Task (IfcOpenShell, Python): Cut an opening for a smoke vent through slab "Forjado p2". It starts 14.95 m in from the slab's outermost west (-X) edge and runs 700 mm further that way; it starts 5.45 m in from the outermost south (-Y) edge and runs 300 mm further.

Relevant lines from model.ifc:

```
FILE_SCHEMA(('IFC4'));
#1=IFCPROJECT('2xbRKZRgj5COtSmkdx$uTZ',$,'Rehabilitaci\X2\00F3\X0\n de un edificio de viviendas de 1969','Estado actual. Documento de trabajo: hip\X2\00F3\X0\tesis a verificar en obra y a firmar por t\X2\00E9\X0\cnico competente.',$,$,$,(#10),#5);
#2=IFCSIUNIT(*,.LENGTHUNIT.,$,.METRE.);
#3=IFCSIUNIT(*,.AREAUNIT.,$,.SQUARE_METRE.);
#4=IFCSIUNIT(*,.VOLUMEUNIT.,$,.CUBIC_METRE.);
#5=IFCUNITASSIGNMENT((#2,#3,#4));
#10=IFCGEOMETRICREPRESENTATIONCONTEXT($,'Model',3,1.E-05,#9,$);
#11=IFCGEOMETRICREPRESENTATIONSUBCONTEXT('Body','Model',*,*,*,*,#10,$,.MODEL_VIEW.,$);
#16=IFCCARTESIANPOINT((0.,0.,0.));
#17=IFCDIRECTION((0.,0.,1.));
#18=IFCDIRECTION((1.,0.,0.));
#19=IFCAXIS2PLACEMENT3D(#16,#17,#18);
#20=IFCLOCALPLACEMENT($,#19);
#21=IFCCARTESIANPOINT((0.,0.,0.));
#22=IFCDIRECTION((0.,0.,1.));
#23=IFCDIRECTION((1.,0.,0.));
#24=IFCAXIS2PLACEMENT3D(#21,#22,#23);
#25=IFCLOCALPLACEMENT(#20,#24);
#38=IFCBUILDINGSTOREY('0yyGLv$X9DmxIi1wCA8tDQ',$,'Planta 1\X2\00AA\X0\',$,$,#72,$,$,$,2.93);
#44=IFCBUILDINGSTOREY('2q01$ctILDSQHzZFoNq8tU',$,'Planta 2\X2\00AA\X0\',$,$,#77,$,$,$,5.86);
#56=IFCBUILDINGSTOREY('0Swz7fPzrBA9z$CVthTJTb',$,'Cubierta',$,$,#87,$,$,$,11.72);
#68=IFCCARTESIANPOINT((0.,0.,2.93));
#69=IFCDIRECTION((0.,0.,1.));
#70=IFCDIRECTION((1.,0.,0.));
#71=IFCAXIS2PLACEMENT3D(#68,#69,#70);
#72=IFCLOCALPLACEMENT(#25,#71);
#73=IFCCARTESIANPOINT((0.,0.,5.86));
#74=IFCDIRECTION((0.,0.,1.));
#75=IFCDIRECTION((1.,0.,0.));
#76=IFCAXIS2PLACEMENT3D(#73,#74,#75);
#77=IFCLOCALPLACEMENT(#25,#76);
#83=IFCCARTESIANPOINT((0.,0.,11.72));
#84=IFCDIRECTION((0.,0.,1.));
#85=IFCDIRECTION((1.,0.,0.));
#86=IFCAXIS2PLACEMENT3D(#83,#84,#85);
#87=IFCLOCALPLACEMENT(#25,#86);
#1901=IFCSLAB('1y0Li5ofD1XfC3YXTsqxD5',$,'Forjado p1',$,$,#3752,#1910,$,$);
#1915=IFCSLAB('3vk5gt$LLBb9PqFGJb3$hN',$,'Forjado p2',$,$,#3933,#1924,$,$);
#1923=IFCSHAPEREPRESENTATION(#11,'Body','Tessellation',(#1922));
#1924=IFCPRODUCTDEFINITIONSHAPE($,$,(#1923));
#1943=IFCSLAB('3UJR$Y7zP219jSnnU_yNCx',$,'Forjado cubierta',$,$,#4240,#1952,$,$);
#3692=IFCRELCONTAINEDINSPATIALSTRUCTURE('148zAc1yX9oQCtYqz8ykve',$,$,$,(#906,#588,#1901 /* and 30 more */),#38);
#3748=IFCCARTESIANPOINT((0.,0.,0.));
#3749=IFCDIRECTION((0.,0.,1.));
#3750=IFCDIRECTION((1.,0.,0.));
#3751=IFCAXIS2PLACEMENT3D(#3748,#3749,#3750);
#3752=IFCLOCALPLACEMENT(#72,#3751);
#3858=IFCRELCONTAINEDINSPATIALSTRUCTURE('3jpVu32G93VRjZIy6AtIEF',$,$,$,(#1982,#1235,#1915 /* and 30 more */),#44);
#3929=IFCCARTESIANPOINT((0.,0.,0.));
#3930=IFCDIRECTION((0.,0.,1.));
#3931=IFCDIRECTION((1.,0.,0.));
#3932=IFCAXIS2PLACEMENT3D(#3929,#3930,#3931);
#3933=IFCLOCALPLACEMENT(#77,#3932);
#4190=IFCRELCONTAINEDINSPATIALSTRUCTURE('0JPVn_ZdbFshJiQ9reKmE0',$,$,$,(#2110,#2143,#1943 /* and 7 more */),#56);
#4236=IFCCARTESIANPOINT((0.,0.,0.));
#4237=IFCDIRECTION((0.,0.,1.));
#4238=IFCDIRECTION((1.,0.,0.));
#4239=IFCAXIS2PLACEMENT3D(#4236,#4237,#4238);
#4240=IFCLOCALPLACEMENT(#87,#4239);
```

```python
import numpy as np
import ifcopenshell
import ifcopenshell.api.feature
import ifcopenshell.api.geometry
import ifcopenshell.api.root
import ifcopenshell.geom
import ifcopenshell.util.placement
import ifcopenshell.util.representation
import ifcopenshell.util.shape
import ifcopenshell.util.unit

model = ifcopenshell.open("model.ifc")
unit_scale = ifcopenshell.util.unit.calculate_unit_scale(model)
settings = ifcopenshell.geom.settings()


def volume(element):
    """Net volume in cubic metres, openings subtracted."""
    shape = ifcopenshell.geom.create_shape(settings, element)
    return ifcopenshell.util.shape.get_volume(shape.geometry)


slab = model.by_id(1915)
before = volume(slab)

# Extent in the slab's own axes, in metres. The edges named are its -X and -Y sides.
slab_shape = ifcopenshell.geom.create_shape(settings, slab)
vertices = ifcopenshell.util.shape.get_vertices(slab_shape.geometry)
x_min, y_min, bottom = vertices.min(axis=0)
top = vertices[:, 2].max()

opening = ifcopenshell.api.root.create_entity(model, ifc_class="IfcOpeningElement", name="Smoke vent opening", predefined_type="OPENING")
context = ifcopenshell.util.representation.get_context(model, "Model", "Body", "MODEL_VIEW")
width, depth = 0.7, 0.3
outline = [(0.0, 0.0), (width, 0.0), (width, depth), (0.0, depth), (0.0, 0.0)]
# Overshoot both faces by 50 mm so the cut is clean.
shape = ifcopenshell.api.geometry.add_slab_representation(
    model, context=context, depth=top - bottom + 0.1, polyline=outline
)
ifcopenshell.api.geometry.assign_representation(model, product=opening, representation=shape)

matrix = ifcopenshell.util.placement.get_local_placement(slab.ObjectPlacement)
matrix[:, 3] = matrix @ np.append(np.array([x_min + 14.95, y_min + 5.45, bottom - 0.05]) / unit_scale, 1.0)
ifcopenshell.api.geometry.edit_object_placement(model, product=opening, matrix=matrix, is_si=False)
ifcopenshell.api.feature.add_feature(model, feature=opening, element=slab)

after = volume(slab)

print(f"slab volume {before:.3f} -> {after:.3f} m3")

model.write("model-out.ifc")
```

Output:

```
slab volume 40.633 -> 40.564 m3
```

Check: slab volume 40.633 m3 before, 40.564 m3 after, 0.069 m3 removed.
